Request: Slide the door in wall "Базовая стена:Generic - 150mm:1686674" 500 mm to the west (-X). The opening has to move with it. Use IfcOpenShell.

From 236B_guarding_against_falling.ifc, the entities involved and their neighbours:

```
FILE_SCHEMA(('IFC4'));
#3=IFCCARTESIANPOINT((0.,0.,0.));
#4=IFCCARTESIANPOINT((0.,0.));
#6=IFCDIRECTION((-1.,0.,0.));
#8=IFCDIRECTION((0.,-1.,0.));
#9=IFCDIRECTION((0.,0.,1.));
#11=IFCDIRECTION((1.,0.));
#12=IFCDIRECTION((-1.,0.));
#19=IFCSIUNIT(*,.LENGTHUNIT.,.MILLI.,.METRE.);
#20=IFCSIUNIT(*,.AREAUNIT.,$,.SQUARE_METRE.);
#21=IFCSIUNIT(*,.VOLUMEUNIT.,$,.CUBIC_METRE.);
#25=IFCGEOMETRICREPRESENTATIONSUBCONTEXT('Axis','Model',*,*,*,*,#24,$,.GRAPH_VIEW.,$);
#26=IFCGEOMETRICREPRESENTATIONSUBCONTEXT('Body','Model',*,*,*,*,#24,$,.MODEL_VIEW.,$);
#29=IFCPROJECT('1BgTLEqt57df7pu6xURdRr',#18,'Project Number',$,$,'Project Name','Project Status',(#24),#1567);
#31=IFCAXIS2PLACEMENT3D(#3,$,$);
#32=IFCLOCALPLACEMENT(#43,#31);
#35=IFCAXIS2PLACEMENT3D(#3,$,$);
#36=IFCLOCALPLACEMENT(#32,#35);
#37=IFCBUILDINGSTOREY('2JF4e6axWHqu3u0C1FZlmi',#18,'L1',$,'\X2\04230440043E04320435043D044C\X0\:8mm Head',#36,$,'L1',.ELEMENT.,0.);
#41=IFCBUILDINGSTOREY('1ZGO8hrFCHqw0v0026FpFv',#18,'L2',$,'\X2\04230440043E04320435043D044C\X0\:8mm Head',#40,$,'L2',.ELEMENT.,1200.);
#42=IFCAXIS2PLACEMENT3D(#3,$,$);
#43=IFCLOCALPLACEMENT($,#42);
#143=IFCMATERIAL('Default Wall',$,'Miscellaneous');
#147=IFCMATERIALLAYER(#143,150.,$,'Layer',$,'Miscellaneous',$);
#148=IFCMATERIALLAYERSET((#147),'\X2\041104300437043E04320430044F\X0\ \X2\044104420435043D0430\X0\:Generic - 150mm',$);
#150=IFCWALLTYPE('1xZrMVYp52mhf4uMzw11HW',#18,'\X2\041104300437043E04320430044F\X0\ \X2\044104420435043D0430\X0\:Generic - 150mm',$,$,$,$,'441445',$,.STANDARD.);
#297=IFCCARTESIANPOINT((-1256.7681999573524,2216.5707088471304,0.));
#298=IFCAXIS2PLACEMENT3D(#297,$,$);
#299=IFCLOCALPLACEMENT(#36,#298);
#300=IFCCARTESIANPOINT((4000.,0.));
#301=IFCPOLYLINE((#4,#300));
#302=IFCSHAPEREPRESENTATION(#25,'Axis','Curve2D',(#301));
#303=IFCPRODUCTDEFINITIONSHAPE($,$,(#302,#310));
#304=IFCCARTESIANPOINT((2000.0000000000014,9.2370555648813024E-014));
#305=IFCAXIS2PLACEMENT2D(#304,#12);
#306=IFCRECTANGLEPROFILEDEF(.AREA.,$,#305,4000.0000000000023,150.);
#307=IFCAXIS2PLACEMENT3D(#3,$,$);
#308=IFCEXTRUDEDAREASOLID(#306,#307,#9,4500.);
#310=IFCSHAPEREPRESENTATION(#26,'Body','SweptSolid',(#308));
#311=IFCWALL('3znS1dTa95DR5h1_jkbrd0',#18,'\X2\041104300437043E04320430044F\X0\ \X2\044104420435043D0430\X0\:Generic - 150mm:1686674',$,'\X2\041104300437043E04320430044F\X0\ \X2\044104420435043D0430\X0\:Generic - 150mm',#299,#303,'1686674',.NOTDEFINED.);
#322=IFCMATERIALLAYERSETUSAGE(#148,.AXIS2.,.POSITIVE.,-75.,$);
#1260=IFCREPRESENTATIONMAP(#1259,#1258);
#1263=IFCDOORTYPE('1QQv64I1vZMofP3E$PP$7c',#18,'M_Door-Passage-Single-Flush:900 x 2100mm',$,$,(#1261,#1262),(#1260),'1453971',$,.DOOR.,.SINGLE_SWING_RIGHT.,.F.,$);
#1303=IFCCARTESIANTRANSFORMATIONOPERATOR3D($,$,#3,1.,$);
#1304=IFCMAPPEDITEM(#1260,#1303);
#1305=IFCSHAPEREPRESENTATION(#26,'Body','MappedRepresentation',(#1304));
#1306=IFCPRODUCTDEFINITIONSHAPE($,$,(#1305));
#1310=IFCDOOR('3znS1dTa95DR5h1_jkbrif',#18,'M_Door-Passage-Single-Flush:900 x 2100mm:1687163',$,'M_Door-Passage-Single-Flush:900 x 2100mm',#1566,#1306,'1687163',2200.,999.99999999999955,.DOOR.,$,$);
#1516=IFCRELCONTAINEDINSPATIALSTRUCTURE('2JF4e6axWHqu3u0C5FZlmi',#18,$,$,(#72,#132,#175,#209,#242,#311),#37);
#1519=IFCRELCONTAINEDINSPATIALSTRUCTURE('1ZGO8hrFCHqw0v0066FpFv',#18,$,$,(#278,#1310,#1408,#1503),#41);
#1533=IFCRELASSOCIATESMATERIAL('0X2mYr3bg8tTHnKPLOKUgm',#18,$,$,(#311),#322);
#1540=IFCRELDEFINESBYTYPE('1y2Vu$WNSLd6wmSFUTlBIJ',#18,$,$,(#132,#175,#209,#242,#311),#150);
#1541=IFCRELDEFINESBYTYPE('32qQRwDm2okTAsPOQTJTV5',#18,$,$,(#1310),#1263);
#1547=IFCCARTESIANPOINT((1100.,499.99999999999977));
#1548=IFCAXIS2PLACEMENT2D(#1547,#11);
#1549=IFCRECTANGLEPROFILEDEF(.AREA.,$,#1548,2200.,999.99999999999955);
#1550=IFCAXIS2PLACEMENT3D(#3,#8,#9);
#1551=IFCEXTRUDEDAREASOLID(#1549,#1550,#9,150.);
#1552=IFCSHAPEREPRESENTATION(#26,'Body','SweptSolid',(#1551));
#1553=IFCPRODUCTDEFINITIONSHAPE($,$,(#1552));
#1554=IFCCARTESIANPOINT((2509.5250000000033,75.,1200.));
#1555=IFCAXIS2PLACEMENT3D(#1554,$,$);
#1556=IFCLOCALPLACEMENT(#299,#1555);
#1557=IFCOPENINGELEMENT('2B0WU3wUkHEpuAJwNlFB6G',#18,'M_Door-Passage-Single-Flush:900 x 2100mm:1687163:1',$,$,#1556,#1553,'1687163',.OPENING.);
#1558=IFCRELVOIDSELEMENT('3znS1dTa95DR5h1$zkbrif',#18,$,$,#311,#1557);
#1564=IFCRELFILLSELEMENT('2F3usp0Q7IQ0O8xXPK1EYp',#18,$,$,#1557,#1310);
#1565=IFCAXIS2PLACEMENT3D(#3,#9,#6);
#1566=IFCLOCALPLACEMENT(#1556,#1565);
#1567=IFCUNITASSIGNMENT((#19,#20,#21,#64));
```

```python
import ifcopenshell
import ifcopenshell.api.geometry
import ifcopenshell.util.placement

model = ifcopenshell.open("236B_guarding_against_falling.ifc")

door = model.by_id(1310)
opening = door.FillsVoids[0].RelatingOpeningElement
wall = opening.VoidsElements[0].RelatingBuildingElement

wall_matrix = ifcopenshell.util.placement.get_local_placement(wall.ObjectPlacement)
shift = wall_matrix[:3, 0] * -500.0
before = ifcopenshell.util.placement.get_local_placement(door.ObjectPlacement)[:3, 3].copy()

# The door is placed relative to its opening, so it follows when the opening moves.
matrix = ifcopenshell.util.placement.get_local_placement(opening.ObjectPlacement)
matrix[:3, 3] += shift
ifcopenshell.api.geometry.edit_object_placement(
    model, product=opening, matrix=matrix, is_si=False, should_transform_children=True
)

after = ifcopenshell.util.placement.get_local_placement(door.ObjectPlacement)[:3, 3]
print("door moved by", (after - before).round(3) + 0.0)

model.write("236B_guarding_against_falling_edited.ifc")
```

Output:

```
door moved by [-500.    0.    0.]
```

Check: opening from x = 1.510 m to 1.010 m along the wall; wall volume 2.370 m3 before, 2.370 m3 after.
